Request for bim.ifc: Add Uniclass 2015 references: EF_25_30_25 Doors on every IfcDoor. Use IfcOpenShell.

First a look at what the model holds.

```python
import ifcopenshell

model = ifcopenshell.open("bim.ifc")
print(model.schema)
print("classifications:", [c.Name for c in model.by_type("IfcClassification")])
for ifc_class in ("IfcDoor", "IfcRoof", "IfcStair", "IfcWall", "IfcWindow"):
    print(ifc_class, len(model.by_type(ifc_class)))
```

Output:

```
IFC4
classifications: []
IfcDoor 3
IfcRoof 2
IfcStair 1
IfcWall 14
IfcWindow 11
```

```python
import ifcopenshell
import ifcopenshell.api.classification

model = ifcopenshell.open("bim.ifc")

system = ifcopenshell.api.classification.add_classification(model, classification="Uniclass 2015")

codes = {
    "IfcDoor": ("EF_25_30_25", "Doors"),
}
for ifc_class, (code, name) in codes.items():
    products = model.by_type(ifc_class)
    ifcopenshell.api.classification.add_reference(
        model, products=products, classification=system, identification=code, name=name
    )
    print(code, len(products))

model.write("bim_rev.ifc")
```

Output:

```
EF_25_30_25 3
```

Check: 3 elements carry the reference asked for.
